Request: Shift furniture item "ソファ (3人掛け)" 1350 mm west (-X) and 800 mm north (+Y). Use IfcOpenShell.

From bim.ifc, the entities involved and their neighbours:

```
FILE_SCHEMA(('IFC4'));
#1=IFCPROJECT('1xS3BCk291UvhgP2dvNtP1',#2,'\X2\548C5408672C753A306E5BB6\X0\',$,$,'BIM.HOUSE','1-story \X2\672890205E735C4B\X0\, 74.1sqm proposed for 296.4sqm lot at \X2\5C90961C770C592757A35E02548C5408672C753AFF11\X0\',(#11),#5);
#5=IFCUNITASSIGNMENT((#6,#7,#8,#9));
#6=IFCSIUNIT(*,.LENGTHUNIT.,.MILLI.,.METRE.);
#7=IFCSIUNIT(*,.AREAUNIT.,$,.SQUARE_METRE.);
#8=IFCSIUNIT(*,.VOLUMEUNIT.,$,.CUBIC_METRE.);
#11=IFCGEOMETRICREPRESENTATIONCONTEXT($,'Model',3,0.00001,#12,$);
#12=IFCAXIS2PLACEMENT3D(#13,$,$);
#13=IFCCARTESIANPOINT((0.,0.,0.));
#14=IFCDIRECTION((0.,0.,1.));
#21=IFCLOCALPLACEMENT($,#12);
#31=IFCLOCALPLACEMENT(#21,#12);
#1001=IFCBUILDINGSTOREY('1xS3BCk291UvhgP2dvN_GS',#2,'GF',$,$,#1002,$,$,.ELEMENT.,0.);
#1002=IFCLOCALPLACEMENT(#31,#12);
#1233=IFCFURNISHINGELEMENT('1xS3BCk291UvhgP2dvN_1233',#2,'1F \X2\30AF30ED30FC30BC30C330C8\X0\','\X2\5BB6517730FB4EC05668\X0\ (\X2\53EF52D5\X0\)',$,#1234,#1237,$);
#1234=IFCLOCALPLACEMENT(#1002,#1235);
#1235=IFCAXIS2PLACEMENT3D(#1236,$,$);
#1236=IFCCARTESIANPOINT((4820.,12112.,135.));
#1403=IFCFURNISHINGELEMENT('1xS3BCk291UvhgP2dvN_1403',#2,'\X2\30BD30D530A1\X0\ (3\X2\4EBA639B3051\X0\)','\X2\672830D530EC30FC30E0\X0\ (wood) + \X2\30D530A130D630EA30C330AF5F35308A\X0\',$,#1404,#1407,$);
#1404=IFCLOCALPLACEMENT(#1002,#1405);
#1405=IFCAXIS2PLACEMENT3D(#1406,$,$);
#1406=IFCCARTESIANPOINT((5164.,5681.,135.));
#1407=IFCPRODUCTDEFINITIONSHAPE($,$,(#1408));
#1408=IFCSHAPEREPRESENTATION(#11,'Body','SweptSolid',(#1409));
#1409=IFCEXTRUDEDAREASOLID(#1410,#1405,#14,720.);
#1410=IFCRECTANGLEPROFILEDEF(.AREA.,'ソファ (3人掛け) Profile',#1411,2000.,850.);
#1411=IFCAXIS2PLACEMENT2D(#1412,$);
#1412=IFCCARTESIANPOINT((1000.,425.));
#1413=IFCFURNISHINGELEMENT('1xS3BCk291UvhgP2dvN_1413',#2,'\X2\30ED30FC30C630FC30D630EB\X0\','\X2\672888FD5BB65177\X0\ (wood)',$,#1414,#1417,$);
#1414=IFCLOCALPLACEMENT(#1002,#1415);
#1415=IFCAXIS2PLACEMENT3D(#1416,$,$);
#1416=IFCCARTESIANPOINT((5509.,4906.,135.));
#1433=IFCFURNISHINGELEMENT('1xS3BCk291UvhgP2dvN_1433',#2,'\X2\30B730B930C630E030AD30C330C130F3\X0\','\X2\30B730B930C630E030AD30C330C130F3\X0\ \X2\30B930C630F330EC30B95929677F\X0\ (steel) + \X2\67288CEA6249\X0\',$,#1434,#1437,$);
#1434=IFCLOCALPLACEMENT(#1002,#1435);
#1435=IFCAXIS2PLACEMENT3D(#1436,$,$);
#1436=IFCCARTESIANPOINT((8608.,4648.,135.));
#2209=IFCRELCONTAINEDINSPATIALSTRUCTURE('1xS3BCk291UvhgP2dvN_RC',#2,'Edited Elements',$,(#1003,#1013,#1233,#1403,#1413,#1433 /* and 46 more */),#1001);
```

```python
import ifcopenshell
import ifcopenshell.api.geometry
import ifcopenshell.util.placement
import ifcopenshell.util.unit

model = ifcopenshell.open("bim.ifc")
unit_scale = ifcopenshell.util.unit.calculate_unit_scale(model)

item = model.by_guid("1xS3BCk291UvhgP2dvN_1403")
matrix = ifcopenshell.util.placement.get_local_placement(item.ObjectPlacement)
matrix[0, 3] -= 1.35 / unit_scale
matrix[1, 3] += 0.8 / unit_scale
ifcopenshell.api.geometry.edit_object_placement(model, product=item, matrix=matrix, is_si=False)

print(ifcopenshell.util.placement.get_local_placement(item.ObjectPlacement).round(3) + 0.0)

model.write("bim_updated.ifc")
```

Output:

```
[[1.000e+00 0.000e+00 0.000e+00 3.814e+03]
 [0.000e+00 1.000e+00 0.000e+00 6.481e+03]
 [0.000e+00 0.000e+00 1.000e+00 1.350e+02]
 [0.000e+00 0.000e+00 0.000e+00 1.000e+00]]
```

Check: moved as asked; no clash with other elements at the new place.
